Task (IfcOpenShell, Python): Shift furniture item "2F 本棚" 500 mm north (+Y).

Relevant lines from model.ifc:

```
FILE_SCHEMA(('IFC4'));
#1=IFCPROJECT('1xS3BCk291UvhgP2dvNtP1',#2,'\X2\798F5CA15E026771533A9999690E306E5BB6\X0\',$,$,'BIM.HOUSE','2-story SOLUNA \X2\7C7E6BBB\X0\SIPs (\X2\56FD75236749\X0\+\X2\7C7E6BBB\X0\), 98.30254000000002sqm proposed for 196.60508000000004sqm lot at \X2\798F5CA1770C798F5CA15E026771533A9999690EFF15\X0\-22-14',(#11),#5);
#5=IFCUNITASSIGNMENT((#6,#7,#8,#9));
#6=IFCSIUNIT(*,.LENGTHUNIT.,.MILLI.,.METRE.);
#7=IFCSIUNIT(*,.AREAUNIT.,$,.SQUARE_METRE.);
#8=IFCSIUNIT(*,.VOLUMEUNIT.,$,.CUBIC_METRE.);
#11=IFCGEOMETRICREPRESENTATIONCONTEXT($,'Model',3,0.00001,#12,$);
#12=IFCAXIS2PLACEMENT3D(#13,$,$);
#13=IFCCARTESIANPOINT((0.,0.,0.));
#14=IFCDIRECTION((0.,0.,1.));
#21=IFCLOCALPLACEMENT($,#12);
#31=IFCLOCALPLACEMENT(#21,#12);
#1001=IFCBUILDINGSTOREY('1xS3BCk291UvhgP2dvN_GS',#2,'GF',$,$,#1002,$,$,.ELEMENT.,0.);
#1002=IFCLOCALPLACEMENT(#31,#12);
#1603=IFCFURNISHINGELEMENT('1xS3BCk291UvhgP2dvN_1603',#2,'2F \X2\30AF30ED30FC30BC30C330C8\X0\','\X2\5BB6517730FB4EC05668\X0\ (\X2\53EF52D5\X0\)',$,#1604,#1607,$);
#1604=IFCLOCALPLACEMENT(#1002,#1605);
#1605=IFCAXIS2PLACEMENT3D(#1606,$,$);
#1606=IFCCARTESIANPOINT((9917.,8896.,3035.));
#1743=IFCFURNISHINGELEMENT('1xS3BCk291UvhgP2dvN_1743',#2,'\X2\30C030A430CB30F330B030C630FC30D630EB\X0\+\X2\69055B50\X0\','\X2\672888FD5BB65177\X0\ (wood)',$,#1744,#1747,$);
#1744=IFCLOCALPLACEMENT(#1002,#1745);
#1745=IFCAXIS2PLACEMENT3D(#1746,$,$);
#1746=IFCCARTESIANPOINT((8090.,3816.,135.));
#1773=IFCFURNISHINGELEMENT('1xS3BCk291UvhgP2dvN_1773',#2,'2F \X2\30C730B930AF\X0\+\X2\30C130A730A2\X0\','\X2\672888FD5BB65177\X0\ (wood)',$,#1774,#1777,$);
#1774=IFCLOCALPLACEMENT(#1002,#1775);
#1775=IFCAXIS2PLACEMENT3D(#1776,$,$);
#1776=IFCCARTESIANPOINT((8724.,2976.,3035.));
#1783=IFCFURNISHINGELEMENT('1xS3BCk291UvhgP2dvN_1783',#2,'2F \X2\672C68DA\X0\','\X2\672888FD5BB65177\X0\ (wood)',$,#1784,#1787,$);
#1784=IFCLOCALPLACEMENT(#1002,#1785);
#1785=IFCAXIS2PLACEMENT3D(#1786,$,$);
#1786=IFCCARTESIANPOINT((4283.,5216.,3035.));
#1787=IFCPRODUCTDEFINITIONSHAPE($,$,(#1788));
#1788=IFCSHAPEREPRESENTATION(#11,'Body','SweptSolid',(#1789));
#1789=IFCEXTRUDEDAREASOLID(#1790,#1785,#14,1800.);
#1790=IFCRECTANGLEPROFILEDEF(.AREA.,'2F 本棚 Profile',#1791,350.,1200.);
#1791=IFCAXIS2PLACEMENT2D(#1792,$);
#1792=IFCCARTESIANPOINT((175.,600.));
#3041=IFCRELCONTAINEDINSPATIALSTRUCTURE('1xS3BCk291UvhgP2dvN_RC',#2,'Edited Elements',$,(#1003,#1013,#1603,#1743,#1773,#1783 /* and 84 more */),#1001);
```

```python
import ifcopenshell
import ifcopenshell.api.geometry
import ifcopenshell.util.placement

model = ifcopenshell.open("model.ifc")

item = model.by_id(1783)
matrix = ifcopenshell.util.placement.get_local_placement(item.ObjectPlacement)
matrix[1, 3] += 500.0
ifcopenshell.api.geometry.edit_object_placement(model, product=item, matrix=matrix, is_si=False)

print(ifcopenshell.util.placement.get_local_placement(item.ObjectPlacement).round(3) + 0.0)

model.write("model_updated.ifc")
```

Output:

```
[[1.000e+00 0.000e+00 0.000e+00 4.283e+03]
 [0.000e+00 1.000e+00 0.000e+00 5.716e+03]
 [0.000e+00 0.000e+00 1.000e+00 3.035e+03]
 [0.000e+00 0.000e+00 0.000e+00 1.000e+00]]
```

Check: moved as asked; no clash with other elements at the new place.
